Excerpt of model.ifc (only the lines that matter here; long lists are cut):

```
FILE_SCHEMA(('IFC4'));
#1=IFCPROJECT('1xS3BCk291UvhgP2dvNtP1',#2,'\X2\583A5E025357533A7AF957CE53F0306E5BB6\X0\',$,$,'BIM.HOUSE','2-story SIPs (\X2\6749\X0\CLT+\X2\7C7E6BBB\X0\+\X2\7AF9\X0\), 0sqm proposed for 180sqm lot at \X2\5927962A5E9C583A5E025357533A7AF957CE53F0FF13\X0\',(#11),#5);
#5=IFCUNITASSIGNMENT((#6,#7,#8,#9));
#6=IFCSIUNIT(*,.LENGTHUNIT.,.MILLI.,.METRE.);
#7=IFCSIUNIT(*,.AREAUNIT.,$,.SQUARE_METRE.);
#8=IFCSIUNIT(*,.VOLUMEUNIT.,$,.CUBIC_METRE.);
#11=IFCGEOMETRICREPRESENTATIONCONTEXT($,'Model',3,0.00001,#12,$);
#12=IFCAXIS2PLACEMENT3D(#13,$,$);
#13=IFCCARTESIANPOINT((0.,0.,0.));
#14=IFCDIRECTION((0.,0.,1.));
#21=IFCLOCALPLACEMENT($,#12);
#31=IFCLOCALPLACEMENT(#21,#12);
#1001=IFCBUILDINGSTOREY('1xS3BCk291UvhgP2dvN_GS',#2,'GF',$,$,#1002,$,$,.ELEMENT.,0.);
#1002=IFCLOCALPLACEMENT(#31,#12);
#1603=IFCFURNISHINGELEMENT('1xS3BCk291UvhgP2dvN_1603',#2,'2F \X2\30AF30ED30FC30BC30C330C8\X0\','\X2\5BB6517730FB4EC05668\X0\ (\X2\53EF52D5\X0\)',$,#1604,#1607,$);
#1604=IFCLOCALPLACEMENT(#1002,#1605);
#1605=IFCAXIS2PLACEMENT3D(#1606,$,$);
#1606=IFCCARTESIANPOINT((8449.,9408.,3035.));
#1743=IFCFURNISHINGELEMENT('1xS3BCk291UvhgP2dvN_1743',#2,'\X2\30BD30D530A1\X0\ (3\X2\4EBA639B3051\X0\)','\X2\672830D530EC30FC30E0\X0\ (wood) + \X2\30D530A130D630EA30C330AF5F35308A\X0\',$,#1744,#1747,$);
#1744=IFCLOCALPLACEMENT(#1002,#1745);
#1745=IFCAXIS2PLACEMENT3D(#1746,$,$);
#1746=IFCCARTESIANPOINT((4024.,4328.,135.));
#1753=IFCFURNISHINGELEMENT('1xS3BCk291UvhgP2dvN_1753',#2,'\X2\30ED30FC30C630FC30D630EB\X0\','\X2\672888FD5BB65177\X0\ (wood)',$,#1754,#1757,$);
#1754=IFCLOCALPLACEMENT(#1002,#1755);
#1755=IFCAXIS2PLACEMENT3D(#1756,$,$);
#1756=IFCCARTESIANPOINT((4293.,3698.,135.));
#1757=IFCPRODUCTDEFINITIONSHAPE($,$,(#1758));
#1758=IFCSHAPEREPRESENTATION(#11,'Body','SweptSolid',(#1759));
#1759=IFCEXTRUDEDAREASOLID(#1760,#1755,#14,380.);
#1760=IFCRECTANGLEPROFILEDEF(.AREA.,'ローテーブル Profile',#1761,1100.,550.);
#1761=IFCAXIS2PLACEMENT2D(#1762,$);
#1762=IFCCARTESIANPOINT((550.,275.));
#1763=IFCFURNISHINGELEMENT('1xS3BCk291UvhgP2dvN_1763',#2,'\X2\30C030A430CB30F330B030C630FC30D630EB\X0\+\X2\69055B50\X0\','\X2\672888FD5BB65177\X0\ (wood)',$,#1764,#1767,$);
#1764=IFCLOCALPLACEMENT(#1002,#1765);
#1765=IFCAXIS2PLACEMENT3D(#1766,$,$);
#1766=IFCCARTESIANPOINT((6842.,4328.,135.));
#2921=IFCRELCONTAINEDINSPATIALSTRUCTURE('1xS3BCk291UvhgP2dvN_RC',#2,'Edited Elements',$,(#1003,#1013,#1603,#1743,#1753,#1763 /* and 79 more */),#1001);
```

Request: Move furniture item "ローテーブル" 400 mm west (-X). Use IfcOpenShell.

```python
import ifcopenshell
import ifcopenshell.api.geometry
import ifcopenshell.util.placement
import ifcopenshell.util.unit

model = ifcopenshell.open("model.ifc")
unit_scale = ifcopenshell.util.unit.calculate_unit_scale(model)

item = model.by_guid("1xS3BCk291UvhgP2dvN_1753")
matrix = ifcopenshell.util.placement.get_local_placement(item.ObjectPlacement)
matrix[0, 3] -= 0.4 / unit_scale
ifcopenshell.api.geometry.edit_object_placement(model, product=item, matrix=matrix, is_si=False)

print(ifcopenshell.util.placement.get_local_placement(item.ObjectPlacement).round(3) + 0.0)

model.write("model_rev.ifc")
```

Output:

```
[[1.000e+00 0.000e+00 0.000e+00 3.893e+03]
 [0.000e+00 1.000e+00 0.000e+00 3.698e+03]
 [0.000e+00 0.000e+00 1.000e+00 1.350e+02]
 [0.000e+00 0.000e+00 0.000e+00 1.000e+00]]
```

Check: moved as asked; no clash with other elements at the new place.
